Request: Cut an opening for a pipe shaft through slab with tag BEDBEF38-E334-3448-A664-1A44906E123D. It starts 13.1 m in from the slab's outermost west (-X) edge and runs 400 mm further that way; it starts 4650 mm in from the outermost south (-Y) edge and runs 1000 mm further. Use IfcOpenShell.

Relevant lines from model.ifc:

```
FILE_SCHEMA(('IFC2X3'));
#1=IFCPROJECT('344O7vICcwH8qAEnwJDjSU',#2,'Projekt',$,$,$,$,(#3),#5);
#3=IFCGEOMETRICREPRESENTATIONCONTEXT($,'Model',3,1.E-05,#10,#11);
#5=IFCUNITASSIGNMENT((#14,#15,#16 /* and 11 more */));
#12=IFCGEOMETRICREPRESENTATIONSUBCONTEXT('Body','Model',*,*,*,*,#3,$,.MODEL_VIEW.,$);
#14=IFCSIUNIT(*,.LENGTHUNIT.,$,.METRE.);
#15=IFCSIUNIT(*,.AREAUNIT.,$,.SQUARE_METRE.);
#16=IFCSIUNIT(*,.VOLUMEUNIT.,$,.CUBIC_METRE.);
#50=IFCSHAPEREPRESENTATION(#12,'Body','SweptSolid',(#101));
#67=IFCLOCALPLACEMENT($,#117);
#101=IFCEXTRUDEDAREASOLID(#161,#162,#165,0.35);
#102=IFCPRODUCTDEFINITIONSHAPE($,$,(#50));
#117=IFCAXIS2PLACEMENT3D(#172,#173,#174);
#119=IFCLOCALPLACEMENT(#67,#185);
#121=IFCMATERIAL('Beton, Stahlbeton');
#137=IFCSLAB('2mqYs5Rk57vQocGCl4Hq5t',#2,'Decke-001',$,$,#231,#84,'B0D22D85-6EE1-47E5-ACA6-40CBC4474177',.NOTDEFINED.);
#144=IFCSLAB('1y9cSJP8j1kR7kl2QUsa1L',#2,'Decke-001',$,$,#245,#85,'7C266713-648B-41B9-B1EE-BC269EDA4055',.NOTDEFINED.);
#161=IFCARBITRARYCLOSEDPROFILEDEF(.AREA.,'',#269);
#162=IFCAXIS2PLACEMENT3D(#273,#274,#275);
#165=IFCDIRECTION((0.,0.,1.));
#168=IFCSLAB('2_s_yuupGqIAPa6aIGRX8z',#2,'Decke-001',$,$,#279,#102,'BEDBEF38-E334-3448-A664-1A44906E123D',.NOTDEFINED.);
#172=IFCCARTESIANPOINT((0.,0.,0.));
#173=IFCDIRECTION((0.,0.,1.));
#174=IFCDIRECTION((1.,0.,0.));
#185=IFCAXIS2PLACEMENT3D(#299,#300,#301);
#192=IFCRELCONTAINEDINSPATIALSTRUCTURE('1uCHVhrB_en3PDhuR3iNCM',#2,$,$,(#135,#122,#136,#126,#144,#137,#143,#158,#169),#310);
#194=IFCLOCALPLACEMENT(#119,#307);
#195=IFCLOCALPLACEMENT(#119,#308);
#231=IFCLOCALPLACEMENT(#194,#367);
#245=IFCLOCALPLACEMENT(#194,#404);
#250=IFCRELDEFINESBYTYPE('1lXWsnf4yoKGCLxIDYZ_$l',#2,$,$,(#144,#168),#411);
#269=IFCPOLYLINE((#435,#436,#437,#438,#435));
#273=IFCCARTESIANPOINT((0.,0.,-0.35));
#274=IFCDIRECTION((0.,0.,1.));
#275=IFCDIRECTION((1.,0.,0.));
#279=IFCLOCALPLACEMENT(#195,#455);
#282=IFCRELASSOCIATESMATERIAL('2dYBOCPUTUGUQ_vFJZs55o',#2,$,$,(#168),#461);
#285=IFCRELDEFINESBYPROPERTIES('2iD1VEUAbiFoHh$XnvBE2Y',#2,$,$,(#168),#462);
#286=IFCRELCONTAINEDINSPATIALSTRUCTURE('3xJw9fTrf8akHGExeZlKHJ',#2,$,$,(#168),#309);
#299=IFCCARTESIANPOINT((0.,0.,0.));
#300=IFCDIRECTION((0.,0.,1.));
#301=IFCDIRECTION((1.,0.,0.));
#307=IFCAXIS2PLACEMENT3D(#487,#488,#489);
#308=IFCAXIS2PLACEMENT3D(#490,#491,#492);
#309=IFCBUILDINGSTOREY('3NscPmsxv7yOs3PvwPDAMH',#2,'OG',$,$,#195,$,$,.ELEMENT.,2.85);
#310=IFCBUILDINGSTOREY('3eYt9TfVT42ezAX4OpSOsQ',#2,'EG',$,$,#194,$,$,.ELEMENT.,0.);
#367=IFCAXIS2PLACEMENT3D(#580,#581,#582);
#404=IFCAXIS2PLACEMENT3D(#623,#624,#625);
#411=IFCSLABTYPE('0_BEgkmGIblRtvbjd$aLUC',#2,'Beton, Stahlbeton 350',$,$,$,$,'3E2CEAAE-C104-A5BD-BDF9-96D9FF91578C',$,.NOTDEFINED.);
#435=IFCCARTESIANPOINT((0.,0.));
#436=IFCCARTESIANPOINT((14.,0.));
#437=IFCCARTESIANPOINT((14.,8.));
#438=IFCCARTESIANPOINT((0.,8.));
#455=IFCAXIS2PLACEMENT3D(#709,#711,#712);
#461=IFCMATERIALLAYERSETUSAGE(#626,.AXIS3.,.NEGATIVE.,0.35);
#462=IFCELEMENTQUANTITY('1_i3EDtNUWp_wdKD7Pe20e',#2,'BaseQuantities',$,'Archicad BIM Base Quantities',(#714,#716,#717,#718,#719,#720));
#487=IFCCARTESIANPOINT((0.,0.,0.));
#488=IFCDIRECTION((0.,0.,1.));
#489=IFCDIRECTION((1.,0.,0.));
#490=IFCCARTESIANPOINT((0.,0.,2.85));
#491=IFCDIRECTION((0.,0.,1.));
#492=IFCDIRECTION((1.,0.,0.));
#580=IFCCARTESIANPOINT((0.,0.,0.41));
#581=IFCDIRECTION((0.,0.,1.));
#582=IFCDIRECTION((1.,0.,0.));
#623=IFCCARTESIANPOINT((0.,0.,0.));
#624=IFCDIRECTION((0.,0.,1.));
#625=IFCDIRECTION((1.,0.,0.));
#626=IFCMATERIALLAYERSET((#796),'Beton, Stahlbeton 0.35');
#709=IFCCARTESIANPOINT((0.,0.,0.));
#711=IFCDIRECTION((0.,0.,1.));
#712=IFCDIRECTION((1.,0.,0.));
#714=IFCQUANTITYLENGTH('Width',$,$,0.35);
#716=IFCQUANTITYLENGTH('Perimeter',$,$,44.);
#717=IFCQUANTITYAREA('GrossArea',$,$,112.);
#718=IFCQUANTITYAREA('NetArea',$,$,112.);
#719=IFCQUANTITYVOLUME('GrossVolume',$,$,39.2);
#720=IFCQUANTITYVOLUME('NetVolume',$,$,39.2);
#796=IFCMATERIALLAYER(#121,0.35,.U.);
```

```python
import numpy as np
import ifcopenshell
import ifcopenshell.api.feature
import ifcopenshell.api.geometry
import ifcopenshell.api.pset
import ifcopenshell.api.root
import ifcopenshell.geom
import ifcopenshell.util.element
import ifcopenshell.util.placement
import ifcopenshell.util.representation
import ifcopenshell.util.shape
import ifcopenshell.util.unit

model = ifcopenshell.open("model.ifc")
unit_scale = ifcopenshell.util.unit.calculate_unit_scale(model)
area_scale = ifcopenshell.util.unit.calculate_unit_scale(model, "AREAUNIT")
volume_scale = ifcopenshell.util.unit.calculate_unit_scale(model, "VOLUMEUNIT")
settings = ifcopenshell.geom.settings()


def volume(element):
    """Net volume in cubic metres, openings subtracted."""
    shape = ifcopenshell.geom.create_shape(settings, element)
    return ifcopenshell.util.shape.get_volume(shape.geometry)


slab = model.by_id(168)
before = volume(slab)

# Extent in the slab's own axes, in metres. The edges named are its -X and -Y sides.
slab_shape = ifcopenshell.geom.create_shape(settings, slab)
vertices = ifcopenshell.util.shape.get_vertices(slab_shape.geometry)
x_min, y_min, bottom = vertices.min(axis=0)
top = vertices[:, 2].max()

opening = ifcopenshell.api.root.create_entity(model, ifc_class="IfcOpeningElement", name="Pipe shaft opening")
context = ifcopenshell.util.representation.get_context(model, "Model", "Body", "MODEL_VIEW")
width, depth = 0.4, 1
outline = [(0.0, 0.0), (width, 0.0), (width, depth), (0.0, depth), (0.0, 0.0)]
# Overshoot both faces by 50 mm so the cut is clean.
shape = ifcopenshell.api.geometry.add_slab_representation(
    model, context=context, depth=top - bottom + 0.1, polyline=outline
)
ifcopenshell.api.geometry.assign_representation(model, product=opening, representation=shape)

matrix = ifcopenshell.util.placement.get_local_placement(slab.ObjectPlacement)
matrix[:, 3] = matrix @ np.append(np.array([x_min + 13.1, y_min + 4.65, bottom - 0.05]) / unit_scale, 1.0)
ifcopenshell.api.geometry.edit_object_placement(model, product=opening, matrix=matrix, is_si=False)
ifcopenshell.api.feature.add_feature(model, feature=opening, element=slab)

after = volume(slab)

# Update the slab's stored quantities.
qto = model.by_id(ifcopenshell.util.element.get_pset(slab, "BaseQuantities", should_inherit=False)["id"])
ifcopenshell.api.pset.edit_qto(model, qto=qto, properties={
    "NetArea": after / (top - bottom) / area_scale,
    "NetVolume": after / volume_scale,
})

print(f"slab volume {before:.3f} -> {after:.3f} m3")

model.write("model-out.ifc")
```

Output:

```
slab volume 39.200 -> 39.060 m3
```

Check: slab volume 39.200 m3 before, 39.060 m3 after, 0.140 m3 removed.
